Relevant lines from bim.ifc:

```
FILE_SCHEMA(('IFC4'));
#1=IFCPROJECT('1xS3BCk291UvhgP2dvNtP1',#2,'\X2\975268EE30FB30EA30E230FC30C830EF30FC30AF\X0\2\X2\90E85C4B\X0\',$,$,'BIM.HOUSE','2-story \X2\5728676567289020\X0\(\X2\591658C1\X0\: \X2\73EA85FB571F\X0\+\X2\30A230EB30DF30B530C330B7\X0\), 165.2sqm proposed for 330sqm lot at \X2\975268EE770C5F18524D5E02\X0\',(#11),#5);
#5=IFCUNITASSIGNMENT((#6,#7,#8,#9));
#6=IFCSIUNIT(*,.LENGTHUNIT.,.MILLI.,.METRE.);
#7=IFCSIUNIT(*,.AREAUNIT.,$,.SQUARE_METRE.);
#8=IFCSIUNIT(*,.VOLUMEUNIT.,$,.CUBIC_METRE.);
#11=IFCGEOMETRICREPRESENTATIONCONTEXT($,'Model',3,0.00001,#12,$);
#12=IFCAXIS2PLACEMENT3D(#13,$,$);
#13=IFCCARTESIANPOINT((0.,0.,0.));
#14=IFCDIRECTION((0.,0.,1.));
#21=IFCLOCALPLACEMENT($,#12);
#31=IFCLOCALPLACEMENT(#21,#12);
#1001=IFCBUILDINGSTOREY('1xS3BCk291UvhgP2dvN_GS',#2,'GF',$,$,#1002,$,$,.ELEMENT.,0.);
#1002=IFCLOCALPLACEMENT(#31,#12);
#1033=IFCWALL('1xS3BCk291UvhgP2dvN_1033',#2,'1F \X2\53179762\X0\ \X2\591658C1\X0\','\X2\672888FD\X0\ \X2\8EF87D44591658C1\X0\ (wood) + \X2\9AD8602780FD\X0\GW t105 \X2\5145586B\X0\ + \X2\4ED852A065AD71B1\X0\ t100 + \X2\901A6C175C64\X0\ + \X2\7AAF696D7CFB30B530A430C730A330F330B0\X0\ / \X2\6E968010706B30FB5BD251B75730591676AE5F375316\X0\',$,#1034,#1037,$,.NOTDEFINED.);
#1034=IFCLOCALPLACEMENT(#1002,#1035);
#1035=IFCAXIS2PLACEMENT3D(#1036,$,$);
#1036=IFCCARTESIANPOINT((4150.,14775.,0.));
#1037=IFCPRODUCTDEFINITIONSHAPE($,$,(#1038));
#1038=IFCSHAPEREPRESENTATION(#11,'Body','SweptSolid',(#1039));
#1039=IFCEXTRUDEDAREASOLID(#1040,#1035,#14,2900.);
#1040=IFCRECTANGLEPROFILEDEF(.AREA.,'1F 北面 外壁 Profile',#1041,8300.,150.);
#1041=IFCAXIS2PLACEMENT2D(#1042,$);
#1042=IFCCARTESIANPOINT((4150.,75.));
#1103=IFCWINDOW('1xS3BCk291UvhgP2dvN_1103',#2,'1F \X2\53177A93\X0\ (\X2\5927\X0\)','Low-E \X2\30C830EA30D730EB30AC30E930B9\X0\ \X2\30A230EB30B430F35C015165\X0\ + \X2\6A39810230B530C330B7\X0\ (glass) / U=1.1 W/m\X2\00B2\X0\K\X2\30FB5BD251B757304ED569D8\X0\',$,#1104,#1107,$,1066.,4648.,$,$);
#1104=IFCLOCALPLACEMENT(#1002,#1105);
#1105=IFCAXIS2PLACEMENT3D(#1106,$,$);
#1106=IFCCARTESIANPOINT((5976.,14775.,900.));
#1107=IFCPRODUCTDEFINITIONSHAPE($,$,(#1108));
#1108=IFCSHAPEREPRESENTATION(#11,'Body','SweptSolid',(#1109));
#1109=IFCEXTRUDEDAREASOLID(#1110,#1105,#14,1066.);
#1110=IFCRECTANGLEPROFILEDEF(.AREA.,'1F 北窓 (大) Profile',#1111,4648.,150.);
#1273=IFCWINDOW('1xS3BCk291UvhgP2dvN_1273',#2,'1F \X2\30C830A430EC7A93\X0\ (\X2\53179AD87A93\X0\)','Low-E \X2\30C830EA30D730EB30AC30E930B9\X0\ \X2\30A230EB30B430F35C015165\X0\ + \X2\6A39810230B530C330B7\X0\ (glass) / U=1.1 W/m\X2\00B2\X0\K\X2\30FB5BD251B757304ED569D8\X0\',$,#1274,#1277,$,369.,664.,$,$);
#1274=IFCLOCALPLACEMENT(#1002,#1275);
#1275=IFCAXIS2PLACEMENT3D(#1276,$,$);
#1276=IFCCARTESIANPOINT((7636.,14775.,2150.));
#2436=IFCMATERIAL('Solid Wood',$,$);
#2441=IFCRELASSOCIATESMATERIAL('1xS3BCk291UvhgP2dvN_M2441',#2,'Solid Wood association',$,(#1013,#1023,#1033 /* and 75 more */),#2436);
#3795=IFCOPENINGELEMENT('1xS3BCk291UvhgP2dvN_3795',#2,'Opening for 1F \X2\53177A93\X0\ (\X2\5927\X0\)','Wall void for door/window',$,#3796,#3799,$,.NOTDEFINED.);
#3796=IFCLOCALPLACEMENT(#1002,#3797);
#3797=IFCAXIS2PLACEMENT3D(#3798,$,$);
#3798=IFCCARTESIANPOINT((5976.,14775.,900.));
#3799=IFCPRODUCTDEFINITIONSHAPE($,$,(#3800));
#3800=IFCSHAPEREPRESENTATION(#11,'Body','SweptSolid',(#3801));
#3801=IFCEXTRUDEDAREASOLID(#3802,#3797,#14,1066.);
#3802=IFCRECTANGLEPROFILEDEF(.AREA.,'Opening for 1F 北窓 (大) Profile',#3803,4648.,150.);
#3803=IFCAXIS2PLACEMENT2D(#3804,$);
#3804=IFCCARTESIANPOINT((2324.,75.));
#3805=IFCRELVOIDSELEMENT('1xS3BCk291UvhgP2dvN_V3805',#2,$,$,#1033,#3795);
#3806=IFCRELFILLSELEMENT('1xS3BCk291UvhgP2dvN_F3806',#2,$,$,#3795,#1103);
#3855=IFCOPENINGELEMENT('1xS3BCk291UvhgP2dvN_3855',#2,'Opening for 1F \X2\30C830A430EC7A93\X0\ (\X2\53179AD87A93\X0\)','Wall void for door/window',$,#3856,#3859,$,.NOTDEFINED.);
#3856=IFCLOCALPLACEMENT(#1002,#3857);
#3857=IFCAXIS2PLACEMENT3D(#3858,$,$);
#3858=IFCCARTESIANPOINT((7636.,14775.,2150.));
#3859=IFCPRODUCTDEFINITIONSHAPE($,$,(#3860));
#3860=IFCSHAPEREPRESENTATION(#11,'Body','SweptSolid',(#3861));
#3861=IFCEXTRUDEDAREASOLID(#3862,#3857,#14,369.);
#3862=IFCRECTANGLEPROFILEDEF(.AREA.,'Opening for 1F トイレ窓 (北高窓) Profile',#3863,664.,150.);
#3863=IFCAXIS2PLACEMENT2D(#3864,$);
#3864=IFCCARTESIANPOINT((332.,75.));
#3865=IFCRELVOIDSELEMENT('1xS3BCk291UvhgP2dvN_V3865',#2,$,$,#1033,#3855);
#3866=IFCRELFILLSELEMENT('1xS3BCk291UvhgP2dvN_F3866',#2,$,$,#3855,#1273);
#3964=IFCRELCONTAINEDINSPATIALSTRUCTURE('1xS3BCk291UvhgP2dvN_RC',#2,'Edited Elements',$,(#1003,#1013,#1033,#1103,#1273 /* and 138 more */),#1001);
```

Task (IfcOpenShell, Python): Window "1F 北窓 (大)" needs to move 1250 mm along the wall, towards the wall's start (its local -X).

```python
import ifcopenshell
import ifcopenshell.api.geometry
import ifcopenshell.util.placement
import ifcopenshell.util.unit

model = ifcopenshell.open("bim.ifc")
unit_scale = ifcopenshell.util.unit.calculate_unit_scale(model)

window = model.by_guid("1xS3BCk291UvhgP2dvN_1103")
opening = window.FillsVoids[0].RelatingOpeningElement
wall = opening.VoidsElements[0].RelatingBuildingElement

wall_matrix = ifcopenshell.util.placement.get_local_placement(wall.ObjectPlacement)
shift = wall_matrix[:3, 0] * -1.25 / unit_scale
before = ifcopenshell.util.placement.get_local_placement(window.ObjectPlacement)[:3, 3].copy()

# The window is not placed relative to its opening, so move both.
for product in (opening, window):
    matrix = ifcopenshell.util.placement.get_local_placement(product.ObjectPlacement)
    matrix[:3, 3] += shift
    ifcopenshell.api.geometry.edit_object_placement(model, product=product, matrix=matrix, is_si=False)

after = ifcopenshell.util.placement.get_local_placement(window.ObjectPlacement)[:3, 3]
print("window moved by", (after - before).round(3) + 0.0)

model.write("bim_v2.ifc")
```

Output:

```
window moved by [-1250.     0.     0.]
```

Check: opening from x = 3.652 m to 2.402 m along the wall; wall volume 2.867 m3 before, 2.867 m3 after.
